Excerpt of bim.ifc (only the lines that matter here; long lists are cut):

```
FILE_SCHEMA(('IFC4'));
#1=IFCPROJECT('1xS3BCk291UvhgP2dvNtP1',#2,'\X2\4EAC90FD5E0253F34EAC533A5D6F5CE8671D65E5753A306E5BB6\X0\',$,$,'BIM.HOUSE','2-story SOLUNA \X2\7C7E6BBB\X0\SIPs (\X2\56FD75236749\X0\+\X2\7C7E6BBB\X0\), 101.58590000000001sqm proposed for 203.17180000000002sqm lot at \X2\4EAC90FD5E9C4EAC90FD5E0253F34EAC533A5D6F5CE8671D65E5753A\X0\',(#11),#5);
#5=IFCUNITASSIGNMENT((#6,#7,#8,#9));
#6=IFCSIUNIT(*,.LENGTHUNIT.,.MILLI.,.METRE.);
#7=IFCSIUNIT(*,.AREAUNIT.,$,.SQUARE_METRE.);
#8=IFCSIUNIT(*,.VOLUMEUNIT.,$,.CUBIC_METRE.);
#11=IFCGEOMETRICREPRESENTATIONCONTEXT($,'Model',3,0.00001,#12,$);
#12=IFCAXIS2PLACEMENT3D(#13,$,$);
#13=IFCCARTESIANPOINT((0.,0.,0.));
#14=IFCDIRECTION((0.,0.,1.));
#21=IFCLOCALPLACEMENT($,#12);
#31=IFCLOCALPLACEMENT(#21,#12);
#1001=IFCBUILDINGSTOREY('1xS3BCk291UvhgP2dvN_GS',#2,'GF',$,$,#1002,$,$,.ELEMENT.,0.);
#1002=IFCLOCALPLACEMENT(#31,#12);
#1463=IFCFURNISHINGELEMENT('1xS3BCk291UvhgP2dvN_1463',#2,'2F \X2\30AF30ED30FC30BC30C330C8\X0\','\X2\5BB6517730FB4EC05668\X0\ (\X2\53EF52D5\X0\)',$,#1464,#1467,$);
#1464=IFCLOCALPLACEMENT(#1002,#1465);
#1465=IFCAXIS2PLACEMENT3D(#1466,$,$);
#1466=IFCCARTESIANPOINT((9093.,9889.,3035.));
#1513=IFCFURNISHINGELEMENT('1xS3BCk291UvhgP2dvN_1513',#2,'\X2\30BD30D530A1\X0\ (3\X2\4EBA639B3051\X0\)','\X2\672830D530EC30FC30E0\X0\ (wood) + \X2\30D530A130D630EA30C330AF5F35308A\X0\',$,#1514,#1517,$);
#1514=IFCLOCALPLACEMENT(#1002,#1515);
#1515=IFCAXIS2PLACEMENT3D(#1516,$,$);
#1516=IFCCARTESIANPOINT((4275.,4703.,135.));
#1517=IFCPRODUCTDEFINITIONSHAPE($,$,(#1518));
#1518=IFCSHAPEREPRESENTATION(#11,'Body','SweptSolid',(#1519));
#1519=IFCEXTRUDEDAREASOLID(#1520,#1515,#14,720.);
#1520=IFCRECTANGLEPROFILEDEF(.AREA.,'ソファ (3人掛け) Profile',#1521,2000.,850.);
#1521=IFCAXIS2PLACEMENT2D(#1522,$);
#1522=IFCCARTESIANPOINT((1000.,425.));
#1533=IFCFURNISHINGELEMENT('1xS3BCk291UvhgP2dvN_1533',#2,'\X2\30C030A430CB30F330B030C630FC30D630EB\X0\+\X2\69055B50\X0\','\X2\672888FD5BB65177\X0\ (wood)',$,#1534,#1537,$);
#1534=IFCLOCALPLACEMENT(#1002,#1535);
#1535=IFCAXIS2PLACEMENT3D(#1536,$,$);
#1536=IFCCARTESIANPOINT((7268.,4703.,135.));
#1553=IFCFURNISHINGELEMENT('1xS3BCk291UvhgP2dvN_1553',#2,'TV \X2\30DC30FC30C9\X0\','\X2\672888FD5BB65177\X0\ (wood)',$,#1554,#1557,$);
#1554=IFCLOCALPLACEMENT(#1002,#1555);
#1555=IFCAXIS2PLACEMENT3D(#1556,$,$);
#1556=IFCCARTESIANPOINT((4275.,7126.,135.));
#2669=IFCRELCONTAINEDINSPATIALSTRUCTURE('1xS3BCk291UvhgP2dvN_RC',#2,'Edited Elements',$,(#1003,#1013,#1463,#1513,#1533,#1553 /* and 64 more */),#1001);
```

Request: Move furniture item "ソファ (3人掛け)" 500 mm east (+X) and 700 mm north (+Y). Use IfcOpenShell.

```python
import ifcopenshell
import ifcopenshell.api.geometry
import ifcopenshell.util.placement

model = ifcopenshell.open("bim.ifc")

item = model.by_guid("1xS3BCk291UvhgP2dvN_1513")
matrix = ifcopenshell.util.placement.get_local_placement(item.ObjectPlacement)
matrix[0, 3] += 500.0
matrix[1, 3] += 700.0
ifcopenshell.api.geometry.edit_object_placement(model, product=item, matrix=matrix, is_si=False)

print(ifcopenshell.util.placement.get_local_placement(item.ObjectPlacement).round(3) + 0.0)

model.write("bim_updated.ifc")
```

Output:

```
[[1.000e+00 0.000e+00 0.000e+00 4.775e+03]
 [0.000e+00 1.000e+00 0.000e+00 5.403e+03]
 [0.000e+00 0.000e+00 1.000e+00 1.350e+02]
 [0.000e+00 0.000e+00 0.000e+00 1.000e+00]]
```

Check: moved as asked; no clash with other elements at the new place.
